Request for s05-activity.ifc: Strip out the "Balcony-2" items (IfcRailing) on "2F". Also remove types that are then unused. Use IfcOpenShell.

First a look at what the model holds.

```python
import ifcopenshell
import ifcopenshell.util.element

model = ifcopenshell.open("s05-activity.ifc")
print(model.schema)
storey = next(s for s in model.by_type("IfcBuildingStorey") if s.Name == "2F")
railings = [e for e in ifcopenshell.util.element.get_decomposition(storey) if e.is_a("IfcRailing")]
seen = {}
for e in railings:
    element_type = ifcopenshell.util.element.get_type(e)
    name = element_type.Name if element_type not in (None, e) else None
    seen[name] = seen.get(name, 0) + 1
for name, count in sorted(seen.items(), key=str):
    print(count, "x", name)
```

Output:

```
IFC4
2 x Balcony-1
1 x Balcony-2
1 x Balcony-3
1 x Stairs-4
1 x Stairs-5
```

```python
import ifcopenshell
import ifcopenshell.api.root
import ifcopenshell.util.element

model = ifcopenshell.open("s05-activity.ifc")

storey = next(s for s in model.by_type("IfcBuildingStorey") if s.Name == "2F")
railings = [e for e in ifcopenshell.util.element.get_decomposition(storey) if e.is_a("IfcRailing")]
targets = [e for e in railings if (t := ifcopenshell.util.element.get_type(e)) not in (None, e) and t.Name == "Balcony-2"]
types = {ifcopenshell.util.element.get_type(e) for e in targets} - {None, *targets}

for e in targets:
    ifcopenshell.api.root.remove_product(model, product=e)
print(len(targets), "removed")

unused = [t for t in types if not ifcopenshell.util.element.get_types(t)]
for t in unused:
    ifcopenshell.api.root.remove_product(model, product=t)
print(len(unused), "unused types removed")

model.write("s05-activity_updated.ifc")
```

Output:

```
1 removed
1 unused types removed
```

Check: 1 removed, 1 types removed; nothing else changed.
